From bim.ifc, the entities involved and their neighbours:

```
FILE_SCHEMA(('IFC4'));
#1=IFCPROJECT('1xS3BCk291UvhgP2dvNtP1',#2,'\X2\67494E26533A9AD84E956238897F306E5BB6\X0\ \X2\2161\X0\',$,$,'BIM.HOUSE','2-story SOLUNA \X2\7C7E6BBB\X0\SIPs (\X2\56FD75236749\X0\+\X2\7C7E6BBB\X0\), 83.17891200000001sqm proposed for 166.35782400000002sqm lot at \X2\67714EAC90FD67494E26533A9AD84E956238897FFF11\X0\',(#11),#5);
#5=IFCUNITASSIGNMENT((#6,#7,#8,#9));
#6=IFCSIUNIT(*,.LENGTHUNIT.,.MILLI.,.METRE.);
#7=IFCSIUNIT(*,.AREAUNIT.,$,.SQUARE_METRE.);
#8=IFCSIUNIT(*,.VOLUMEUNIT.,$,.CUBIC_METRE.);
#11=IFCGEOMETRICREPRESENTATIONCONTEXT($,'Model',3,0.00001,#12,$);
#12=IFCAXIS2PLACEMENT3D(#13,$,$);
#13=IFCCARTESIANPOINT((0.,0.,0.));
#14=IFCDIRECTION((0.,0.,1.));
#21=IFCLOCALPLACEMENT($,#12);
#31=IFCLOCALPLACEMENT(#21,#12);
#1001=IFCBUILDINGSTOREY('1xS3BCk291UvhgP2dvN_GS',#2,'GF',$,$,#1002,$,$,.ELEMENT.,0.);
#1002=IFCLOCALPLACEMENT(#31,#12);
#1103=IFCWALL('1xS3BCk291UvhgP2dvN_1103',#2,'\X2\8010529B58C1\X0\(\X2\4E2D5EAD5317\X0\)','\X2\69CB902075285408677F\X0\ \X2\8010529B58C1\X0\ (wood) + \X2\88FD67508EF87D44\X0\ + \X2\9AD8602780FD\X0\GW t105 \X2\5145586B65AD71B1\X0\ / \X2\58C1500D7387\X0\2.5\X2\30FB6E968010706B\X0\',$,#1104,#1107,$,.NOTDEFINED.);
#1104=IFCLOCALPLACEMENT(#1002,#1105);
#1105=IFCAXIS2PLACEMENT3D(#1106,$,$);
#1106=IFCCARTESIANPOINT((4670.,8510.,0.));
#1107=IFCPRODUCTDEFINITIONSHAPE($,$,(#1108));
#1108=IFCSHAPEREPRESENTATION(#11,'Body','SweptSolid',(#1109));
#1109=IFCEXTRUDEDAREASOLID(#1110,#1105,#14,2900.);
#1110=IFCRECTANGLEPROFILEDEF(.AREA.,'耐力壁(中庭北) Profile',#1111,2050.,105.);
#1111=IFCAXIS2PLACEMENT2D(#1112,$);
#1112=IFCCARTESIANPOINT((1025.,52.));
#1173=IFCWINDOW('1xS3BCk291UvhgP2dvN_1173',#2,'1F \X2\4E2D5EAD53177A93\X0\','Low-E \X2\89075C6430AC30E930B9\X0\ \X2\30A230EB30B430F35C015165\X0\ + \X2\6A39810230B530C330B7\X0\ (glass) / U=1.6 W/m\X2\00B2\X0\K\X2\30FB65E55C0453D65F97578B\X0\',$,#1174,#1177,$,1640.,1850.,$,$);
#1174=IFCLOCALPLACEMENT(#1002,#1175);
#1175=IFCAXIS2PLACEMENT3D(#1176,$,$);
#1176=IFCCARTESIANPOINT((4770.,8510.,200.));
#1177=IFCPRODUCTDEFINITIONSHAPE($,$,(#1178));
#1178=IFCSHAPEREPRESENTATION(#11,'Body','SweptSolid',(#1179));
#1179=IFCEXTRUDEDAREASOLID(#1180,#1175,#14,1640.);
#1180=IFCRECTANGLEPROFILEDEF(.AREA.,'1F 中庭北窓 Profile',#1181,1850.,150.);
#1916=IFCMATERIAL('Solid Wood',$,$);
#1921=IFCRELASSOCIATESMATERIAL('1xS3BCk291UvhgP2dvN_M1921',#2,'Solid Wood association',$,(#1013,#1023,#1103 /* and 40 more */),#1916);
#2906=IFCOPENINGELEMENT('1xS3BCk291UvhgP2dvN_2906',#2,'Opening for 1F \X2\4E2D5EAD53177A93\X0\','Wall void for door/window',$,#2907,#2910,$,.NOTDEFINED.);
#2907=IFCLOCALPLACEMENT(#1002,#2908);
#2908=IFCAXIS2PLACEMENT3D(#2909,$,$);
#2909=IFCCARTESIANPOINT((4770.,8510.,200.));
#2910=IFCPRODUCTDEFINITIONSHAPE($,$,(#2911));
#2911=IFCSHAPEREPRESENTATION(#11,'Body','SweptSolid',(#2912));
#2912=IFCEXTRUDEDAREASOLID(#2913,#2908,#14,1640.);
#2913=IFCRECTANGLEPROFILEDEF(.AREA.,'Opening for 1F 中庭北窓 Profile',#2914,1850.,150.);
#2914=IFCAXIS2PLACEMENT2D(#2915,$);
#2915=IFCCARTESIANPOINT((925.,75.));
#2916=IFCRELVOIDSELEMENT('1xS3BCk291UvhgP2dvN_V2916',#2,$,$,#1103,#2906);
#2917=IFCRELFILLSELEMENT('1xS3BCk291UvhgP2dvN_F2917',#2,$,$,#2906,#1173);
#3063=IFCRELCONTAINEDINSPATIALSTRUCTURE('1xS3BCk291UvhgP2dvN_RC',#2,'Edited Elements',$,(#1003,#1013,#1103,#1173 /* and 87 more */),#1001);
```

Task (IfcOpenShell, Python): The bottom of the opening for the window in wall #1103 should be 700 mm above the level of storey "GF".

```python
import numpy as np
import ifcopenshell
import ifcopenshell.api.geometry
import ifcopenshell.geom
import ifcopenshell.util.element
import ifcopenshell.util.placement
import ifcopenshell.util.shape
import ifcopenshell.util.unit

model = ifcopenshell.open("bim.ifc")
unit_scale = ifcopenshell.util.unit.calculate_unit_scale(model)

window = model.by_id(1173)
opening = window.FillsVoids[0].RelatingOpeningElement
storey = ifcopenshell.util.element.get_container(window, ifc_class="IfcBuildingStorey")
level = ifcopenshell.util.placement.get_local_placement(storey.ObjectPlacement)[2, 3]

# The opening's origin need not be at the sill, so measure its lowest point.
shape = ifcopenshell.geom.create_shape(ifcopenshell.geom.settings(), opening)
bottom = ifcopenshell.util.shape.get_shape_bottom_elevation(shape, shape.geometry) / unit_scale
dz = level + 0.7 / unit_scale - bottom

shift = np.array([0.0, 0.0, dz])
# The window is not placed relative to its opening, so move both.
for product in (opening, window):
    matrix = ifcopenshell.util.placement.get_local_placement(product.ObjectPlacement)
    matrix[:3, 3] += shift
    ifcopenshell.api.geometry.edit_object_placement(model, product=product, matrix=matrix, is_si=False)

print(f"moved by {dz * unit_scale:+.3f} m")

model.write("bim_updated.ifc")
```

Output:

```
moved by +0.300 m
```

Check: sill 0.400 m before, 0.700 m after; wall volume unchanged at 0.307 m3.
